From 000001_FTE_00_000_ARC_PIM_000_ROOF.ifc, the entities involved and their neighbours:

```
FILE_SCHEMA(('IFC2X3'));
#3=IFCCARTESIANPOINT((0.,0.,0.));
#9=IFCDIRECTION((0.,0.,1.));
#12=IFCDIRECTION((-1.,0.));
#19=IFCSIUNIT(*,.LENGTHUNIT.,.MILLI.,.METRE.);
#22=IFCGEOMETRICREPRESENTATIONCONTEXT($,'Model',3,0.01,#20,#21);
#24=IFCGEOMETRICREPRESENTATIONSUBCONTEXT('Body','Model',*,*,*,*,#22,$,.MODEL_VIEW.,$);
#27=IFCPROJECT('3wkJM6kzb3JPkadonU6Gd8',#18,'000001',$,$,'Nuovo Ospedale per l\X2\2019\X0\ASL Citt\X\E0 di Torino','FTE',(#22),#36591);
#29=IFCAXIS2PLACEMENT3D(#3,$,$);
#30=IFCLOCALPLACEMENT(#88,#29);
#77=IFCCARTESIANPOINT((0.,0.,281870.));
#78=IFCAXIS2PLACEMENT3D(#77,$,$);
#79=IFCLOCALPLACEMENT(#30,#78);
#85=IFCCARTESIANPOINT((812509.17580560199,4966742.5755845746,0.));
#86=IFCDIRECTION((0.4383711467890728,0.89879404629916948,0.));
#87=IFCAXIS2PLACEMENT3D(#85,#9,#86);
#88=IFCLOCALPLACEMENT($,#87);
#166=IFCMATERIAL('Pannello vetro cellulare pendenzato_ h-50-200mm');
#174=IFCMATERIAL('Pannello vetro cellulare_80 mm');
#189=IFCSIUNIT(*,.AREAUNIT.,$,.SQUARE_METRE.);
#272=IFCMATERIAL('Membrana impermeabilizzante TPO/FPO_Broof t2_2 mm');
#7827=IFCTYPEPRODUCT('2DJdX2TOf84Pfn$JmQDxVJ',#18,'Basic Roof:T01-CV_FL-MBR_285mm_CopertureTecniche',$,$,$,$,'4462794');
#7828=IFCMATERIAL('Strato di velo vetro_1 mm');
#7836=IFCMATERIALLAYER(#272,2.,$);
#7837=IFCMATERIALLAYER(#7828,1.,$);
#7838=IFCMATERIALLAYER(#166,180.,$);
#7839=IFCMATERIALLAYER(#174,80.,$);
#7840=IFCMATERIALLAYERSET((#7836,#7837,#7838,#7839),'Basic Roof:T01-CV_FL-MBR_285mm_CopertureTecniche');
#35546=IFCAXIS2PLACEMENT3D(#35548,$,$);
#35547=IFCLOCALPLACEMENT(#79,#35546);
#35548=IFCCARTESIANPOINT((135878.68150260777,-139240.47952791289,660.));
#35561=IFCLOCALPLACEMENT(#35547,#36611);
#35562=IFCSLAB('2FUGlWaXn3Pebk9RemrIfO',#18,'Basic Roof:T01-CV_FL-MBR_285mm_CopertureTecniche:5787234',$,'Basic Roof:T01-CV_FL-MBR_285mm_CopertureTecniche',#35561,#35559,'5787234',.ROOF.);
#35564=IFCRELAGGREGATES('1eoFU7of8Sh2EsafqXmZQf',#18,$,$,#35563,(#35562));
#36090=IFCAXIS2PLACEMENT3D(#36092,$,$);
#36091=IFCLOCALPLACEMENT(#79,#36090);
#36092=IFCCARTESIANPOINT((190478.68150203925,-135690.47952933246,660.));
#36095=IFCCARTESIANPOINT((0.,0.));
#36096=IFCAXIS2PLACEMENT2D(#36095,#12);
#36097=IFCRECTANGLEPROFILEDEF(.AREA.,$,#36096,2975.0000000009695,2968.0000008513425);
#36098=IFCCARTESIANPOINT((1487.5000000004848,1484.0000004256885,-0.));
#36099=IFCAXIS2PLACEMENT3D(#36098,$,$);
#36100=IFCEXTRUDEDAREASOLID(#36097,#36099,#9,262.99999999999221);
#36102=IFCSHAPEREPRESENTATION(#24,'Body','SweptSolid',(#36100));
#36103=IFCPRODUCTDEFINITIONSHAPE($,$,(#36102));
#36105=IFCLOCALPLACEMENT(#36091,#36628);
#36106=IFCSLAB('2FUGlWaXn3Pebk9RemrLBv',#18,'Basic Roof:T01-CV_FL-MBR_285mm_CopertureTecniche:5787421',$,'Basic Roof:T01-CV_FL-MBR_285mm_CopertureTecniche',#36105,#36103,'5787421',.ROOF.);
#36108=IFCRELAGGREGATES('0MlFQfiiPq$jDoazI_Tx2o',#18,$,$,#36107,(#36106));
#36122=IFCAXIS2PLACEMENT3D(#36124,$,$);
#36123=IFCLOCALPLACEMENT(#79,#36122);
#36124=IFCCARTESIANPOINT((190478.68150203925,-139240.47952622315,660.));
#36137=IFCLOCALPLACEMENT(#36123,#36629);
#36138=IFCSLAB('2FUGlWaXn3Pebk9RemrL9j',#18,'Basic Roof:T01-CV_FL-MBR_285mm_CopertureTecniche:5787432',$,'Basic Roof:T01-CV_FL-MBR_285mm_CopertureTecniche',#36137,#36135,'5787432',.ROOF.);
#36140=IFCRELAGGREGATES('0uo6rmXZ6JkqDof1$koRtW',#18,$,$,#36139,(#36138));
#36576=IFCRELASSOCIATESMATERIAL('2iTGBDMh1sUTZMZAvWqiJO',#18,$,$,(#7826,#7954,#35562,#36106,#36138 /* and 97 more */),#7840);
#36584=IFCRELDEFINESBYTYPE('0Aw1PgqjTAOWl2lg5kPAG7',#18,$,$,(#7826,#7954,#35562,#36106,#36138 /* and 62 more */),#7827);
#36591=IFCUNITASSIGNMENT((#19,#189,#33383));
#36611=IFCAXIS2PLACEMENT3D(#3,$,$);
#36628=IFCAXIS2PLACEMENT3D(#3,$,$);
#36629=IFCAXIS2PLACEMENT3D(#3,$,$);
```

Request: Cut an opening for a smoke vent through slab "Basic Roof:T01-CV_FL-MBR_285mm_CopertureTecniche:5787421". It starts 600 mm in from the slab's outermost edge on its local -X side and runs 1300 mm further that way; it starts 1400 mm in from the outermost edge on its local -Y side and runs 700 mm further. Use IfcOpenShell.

```python
import numpy as np
import ifcopenshell
import ifcopenshell.api.feature
import ifcopenshell.api.geometry
import ifcopenshell.api.root
import ifcopenshell.geom
import ifcopenshell.util.placement
import ifcopenshell.util.representation
import ifcopenshell.util.shape
import ifcopenshell.util.unit

model = ifcopenshell.open("000001_FTE_00_000_ARC_PIM_000_ROOF.ifc")
unit_scale = ifcopenshell.util.unit.calculate_unit_scale(model)
settings = ifcopenshell.geom.settings()


def volume(element):
    """Net volume in cubic metres, openings subtracted."""
    shape = ifcopenshell.geom.create_shape(settings, element)
    return ifcopenshell.util.shape.get_volume(shape.geometry)


slab = model.by_guid("2FUGlWaXn3Pebk9RemrLBv")
before = volume(slab)

# Extent in the slab's own axes, in metres. The edges named are its -X and -Y sides.
slab_shape = ifcopenshell.geom.create_shape(settings, slab)
vertices = ifcopenshell.util.shape.get_vertices(slab_shape.geometry)
x_min, y_min, bottom = vertices.min(axis=0)
top = vertices[:, 2].max()

opening = ifcopenshell.api.root.create_entity(model, ifc_class="IfcOpeningElement", name="Smoke vent opening")
context = ifcopenshell.util.representation.get_context(model, "Model", "Body", "MODEL_VIEW")
width, depth = 1.3, 0.7
outline = [(0.0, 0.0), (width, 0.0), (width, depth), (0.0, depth), (0.0, 0.0)]
# Overshoot both faces by 50 mm so the cut is clean.
shape = ifcopenshell.api.geometry.add_slab_representation(
    model, context=context, depth=top - bottom + 0.1, polyline=outline
)
ifcopenshell.api.geometry.assign_representation(model, product=opening, representation=shape)

matrix = ifcopenshell.util.placement.get_local_placement(slab.ObjectPlacement)
matrix[:, 3] = matrix @ np.append(np.array([x_min + 0.6, y_min + 1.4, bottom - 0.05]) / unit_scale, 1.0)
ifcopenshell.api.geometry.edit_object_placement(model, product=opening, matrix=matrix, is_si=False)
ifcopenshell.api.feature.add_feature(model, feature=opening, element=slab)

after = volume(slab)

print(f"slab volume {before:.3f} -> {after:.3f} m3")

model.write("000001_FTE_00_000_ARC_PIM_000_ROOF_updated.ifc")
```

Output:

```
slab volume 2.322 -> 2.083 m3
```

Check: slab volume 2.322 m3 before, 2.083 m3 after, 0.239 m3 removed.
